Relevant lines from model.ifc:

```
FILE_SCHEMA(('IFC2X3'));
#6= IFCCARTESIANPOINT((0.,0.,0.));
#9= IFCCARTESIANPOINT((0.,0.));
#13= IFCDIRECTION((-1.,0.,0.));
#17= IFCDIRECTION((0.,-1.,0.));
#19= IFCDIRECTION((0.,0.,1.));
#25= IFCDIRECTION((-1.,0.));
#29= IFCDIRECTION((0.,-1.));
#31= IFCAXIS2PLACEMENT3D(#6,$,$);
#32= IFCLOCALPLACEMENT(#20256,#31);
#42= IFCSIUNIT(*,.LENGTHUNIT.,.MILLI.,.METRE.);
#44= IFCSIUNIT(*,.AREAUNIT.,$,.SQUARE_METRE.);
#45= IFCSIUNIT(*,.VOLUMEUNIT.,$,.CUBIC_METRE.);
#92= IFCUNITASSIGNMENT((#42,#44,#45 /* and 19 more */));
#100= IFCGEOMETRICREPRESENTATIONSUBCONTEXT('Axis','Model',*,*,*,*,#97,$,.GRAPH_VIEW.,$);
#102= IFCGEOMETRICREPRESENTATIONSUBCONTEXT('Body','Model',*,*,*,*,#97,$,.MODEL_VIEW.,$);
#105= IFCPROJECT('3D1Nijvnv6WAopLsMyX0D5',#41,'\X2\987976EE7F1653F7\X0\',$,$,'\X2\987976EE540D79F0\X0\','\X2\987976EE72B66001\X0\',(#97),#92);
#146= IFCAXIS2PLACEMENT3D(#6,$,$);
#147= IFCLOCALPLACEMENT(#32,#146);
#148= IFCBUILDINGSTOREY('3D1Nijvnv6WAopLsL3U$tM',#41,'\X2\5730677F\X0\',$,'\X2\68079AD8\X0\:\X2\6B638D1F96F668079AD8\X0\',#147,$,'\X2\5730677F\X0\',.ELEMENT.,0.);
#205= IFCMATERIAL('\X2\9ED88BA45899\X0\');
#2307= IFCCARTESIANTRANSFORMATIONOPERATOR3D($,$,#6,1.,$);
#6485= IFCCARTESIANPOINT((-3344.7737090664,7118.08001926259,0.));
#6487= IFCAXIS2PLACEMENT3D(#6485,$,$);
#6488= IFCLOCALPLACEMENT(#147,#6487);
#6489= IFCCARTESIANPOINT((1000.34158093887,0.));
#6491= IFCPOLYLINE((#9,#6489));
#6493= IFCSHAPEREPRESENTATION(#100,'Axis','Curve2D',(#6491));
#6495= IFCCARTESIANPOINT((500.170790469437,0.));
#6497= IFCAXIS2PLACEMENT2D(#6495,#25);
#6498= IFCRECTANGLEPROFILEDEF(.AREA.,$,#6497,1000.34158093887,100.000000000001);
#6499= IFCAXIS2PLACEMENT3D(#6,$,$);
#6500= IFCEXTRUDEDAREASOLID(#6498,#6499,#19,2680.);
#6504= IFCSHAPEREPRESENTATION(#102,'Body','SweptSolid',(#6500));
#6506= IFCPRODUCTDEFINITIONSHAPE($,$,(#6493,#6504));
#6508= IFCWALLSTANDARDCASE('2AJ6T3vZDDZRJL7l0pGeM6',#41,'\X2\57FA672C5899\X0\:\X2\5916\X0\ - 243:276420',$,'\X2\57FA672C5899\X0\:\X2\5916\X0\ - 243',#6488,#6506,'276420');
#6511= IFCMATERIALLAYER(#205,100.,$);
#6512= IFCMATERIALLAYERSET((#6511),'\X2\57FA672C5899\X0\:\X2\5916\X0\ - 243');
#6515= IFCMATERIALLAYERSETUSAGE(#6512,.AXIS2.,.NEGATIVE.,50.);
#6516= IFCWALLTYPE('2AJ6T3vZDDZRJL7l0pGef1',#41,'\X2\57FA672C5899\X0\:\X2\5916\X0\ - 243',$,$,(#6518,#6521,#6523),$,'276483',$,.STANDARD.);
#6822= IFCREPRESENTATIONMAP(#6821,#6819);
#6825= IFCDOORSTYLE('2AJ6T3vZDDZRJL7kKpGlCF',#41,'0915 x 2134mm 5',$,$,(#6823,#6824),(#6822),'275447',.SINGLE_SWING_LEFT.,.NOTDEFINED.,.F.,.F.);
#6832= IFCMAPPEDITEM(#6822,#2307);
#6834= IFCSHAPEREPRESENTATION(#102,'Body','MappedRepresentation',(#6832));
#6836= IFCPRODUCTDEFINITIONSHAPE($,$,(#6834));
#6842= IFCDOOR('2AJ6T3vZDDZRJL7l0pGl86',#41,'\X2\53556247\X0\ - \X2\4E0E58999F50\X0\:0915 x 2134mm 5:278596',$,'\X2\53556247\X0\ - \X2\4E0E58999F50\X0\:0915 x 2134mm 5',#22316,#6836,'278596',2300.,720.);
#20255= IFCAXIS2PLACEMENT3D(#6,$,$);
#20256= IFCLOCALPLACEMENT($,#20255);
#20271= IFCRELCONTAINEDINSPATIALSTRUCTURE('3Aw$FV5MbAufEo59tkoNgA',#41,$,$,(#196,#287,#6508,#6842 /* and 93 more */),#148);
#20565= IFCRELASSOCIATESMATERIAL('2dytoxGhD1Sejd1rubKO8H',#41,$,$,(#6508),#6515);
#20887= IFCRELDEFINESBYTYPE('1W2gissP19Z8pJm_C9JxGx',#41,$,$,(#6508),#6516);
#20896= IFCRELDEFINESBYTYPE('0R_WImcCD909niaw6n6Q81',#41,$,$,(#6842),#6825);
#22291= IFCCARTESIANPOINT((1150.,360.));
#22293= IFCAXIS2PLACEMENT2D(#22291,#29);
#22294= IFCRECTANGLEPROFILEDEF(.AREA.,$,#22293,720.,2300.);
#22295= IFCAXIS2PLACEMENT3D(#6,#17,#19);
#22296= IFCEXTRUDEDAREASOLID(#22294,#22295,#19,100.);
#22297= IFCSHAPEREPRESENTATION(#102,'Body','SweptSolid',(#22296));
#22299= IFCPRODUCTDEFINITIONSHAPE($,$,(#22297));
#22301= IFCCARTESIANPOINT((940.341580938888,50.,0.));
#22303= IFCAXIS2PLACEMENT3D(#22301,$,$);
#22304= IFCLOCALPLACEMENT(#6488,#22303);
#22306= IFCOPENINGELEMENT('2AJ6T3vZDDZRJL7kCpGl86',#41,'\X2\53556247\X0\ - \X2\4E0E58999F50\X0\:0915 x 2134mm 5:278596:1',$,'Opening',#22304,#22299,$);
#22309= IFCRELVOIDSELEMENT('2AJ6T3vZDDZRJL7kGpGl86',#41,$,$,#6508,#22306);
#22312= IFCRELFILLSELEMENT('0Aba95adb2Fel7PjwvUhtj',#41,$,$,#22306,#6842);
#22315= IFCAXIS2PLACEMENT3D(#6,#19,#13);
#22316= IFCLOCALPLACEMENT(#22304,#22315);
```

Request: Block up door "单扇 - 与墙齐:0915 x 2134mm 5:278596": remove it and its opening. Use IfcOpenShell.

```python
import ifcopenshell
import ifcopenshell.api.feature
import ifcopenshell.api.root
import ifcopenshell.geom
import ifcopenshell.util.shape

model = ifcopenshell.open("model.ifc")
settings = ifcopenshell.geom.settings()


def volume(element):
    """Net volume in cubic metres, openings subtracted."""
    shape = ifcopenshell.geom.create_shape(settings, element)
    return ifcopenshell.util.shape.get_volume(shape.geometry)


door = model.by_guid("2AJ6T3vZDDZRJL7l0pGl86")
opening = door.FillsVoids[0].RelatingOpeningElement
wall = opening.VoidsElements[0].RelatingBuildingElement
before = volume(wall)

ifcopenshell.api.root.remove_product(model, product=door)
ifcopenshell.api.feature.remove_feature(model, feature=opening)

after = volume(wall)

print(f"wall volume {before:.3f} -> {after:.3f} m3")

model.write("model_rev.ifc")
```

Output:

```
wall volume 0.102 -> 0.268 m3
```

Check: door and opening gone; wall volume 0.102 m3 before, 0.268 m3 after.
